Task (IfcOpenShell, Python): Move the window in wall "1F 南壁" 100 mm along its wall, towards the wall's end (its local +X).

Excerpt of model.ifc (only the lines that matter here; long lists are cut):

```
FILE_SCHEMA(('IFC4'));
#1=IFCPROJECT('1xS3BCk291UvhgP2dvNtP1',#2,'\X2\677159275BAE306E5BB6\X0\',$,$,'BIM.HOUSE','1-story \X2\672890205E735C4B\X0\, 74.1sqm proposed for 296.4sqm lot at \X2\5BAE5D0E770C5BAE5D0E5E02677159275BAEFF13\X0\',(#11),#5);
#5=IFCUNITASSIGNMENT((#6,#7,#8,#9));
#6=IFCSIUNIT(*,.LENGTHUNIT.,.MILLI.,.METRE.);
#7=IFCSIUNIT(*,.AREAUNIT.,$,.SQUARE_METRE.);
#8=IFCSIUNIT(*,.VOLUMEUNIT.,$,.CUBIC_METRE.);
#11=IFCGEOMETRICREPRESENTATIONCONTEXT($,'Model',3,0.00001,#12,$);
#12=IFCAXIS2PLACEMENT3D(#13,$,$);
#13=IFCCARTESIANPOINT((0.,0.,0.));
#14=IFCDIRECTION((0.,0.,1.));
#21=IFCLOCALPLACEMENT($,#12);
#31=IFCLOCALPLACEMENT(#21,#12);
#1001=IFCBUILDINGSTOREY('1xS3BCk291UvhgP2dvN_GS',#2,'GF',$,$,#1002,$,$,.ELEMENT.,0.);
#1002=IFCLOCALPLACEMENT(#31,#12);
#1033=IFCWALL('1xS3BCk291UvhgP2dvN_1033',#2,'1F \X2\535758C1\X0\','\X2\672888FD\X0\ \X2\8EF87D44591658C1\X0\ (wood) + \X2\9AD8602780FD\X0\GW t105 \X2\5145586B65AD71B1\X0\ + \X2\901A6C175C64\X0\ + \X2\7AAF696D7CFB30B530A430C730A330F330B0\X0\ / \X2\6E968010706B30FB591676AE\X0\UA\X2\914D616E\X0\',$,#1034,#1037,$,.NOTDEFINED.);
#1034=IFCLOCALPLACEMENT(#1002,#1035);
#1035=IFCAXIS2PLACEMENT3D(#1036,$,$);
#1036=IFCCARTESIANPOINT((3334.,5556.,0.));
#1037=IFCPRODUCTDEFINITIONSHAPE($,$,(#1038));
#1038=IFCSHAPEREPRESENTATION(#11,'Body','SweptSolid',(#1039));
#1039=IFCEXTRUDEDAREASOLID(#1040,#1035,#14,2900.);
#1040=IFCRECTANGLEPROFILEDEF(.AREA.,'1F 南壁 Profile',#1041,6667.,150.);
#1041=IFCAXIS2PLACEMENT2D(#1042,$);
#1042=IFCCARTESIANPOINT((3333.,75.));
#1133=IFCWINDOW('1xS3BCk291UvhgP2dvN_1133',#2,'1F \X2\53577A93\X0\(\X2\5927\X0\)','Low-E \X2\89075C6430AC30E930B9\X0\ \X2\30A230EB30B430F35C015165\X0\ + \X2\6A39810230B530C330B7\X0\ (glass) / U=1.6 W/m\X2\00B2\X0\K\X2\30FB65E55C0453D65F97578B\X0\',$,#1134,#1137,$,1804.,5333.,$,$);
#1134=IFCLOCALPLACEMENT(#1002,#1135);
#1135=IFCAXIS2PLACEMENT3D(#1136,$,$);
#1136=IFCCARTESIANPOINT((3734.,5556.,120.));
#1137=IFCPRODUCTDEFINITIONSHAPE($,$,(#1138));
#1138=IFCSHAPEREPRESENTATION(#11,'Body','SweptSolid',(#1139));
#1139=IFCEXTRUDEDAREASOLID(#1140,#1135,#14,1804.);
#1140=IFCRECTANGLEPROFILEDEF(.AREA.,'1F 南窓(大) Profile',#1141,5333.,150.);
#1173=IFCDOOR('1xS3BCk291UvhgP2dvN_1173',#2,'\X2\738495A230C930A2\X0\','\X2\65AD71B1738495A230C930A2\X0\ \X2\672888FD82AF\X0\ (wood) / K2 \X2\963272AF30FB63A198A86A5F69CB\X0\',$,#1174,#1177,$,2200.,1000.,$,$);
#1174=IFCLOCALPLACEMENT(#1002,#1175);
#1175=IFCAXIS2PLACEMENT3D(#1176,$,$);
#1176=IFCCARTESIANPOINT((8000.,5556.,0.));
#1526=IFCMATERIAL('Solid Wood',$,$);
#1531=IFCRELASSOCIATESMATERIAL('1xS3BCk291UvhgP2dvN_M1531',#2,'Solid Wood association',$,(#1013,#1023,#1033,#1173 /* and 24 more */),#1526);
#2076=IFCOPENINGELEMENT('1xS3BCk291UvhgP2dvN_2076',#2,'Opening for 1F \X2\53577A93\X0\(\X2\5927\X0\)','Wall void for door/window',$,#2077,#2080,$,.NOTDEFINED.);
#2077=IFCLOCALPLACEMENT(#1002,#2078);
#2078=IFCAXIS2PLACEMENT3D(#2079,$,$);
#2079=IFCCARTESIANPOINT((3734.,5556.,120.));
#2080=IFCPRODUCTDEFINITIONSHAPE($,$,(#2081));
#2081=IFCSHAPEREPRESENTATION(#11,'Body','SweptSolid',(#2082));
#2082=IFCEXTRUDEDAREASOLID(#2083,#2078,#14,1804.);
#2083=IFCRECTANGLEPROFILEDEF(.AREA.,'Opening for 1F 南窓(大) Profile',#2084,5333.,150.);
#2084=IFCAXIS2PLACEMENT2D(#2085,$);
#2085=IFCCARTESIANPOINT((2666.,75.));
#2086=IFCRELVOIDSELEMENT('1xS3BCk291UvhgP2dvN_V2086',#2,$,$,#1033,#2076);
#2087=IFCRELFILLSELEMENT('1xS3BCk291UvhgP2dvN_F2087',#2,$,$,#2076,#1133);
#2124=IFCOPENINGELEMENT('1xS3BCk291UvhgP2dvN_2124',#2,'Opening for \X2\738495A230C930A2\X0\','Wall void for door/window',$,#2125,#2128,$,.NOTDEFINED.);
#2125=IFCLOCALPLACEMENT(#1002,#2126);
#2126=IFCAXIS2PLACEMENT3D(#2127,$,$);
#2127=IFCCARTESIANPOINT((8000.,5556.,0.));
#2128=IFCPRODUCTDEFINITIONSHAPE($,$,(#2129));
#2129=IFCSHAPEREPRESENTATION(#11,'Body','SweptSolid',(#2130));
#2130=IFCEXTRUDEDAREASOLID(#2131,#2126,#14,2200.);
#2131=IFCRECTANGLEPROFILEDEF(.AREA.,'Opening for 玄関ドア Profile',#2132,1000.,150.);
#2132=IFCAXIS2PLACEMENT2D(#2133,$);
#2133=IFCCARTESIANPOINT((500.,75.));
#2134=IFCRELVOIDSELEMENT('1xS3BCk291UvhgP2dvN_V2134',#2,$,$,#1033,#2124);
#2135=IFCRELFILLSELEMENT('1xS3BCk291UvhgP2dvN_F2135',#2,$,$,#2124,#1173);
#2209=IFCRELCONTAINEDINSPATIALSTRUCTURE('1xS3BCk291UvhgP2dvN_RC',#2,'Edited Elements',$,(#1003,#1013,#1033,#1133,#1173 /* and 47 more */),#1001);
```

```python
import ifcopenshell
import ifcopenshell.api.geometry
import ifcopenshell.util.placement

model = ifcopenshell.open("model.ifc")

window = model.by_id(1133)
opening = window.FillsVoids[0].RelatingOpeningElement
wall = opening.VoidsElements[0].RelatingBuildingElement

wall_matrix = ifcopenshell.util.placement.get_local_placement(wall.ObjectPlacement)
shift = wall_matrix[:3, 0] * 100.0
before = ifcopenshell.util.placement.get_local_placement(window.ObjectPlacement)[:3, 3].copy()

# The window is not placed relative to its opening, so move both.
for product in (opening, window):
    matrix = ifcopenshell.util.placement.get_local_placement(product.ObjectPlacement)
    matrix[:3, 3] += shift
    ifcopenshell.api.geometry.edit_object_placement(model, product=product, matrix=matrix, is_si=False)

after = ifcopenshell.util.placement.get_local_placement(window.ObjectPlacement)[:3, 3]
print("window moved by", (after - before).round(3) + 0.0)

model.write("model_v2.ifc")
```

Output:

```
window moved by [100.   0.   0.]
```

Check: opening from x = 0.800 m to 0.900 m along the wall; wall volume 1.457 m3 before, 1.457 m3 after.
